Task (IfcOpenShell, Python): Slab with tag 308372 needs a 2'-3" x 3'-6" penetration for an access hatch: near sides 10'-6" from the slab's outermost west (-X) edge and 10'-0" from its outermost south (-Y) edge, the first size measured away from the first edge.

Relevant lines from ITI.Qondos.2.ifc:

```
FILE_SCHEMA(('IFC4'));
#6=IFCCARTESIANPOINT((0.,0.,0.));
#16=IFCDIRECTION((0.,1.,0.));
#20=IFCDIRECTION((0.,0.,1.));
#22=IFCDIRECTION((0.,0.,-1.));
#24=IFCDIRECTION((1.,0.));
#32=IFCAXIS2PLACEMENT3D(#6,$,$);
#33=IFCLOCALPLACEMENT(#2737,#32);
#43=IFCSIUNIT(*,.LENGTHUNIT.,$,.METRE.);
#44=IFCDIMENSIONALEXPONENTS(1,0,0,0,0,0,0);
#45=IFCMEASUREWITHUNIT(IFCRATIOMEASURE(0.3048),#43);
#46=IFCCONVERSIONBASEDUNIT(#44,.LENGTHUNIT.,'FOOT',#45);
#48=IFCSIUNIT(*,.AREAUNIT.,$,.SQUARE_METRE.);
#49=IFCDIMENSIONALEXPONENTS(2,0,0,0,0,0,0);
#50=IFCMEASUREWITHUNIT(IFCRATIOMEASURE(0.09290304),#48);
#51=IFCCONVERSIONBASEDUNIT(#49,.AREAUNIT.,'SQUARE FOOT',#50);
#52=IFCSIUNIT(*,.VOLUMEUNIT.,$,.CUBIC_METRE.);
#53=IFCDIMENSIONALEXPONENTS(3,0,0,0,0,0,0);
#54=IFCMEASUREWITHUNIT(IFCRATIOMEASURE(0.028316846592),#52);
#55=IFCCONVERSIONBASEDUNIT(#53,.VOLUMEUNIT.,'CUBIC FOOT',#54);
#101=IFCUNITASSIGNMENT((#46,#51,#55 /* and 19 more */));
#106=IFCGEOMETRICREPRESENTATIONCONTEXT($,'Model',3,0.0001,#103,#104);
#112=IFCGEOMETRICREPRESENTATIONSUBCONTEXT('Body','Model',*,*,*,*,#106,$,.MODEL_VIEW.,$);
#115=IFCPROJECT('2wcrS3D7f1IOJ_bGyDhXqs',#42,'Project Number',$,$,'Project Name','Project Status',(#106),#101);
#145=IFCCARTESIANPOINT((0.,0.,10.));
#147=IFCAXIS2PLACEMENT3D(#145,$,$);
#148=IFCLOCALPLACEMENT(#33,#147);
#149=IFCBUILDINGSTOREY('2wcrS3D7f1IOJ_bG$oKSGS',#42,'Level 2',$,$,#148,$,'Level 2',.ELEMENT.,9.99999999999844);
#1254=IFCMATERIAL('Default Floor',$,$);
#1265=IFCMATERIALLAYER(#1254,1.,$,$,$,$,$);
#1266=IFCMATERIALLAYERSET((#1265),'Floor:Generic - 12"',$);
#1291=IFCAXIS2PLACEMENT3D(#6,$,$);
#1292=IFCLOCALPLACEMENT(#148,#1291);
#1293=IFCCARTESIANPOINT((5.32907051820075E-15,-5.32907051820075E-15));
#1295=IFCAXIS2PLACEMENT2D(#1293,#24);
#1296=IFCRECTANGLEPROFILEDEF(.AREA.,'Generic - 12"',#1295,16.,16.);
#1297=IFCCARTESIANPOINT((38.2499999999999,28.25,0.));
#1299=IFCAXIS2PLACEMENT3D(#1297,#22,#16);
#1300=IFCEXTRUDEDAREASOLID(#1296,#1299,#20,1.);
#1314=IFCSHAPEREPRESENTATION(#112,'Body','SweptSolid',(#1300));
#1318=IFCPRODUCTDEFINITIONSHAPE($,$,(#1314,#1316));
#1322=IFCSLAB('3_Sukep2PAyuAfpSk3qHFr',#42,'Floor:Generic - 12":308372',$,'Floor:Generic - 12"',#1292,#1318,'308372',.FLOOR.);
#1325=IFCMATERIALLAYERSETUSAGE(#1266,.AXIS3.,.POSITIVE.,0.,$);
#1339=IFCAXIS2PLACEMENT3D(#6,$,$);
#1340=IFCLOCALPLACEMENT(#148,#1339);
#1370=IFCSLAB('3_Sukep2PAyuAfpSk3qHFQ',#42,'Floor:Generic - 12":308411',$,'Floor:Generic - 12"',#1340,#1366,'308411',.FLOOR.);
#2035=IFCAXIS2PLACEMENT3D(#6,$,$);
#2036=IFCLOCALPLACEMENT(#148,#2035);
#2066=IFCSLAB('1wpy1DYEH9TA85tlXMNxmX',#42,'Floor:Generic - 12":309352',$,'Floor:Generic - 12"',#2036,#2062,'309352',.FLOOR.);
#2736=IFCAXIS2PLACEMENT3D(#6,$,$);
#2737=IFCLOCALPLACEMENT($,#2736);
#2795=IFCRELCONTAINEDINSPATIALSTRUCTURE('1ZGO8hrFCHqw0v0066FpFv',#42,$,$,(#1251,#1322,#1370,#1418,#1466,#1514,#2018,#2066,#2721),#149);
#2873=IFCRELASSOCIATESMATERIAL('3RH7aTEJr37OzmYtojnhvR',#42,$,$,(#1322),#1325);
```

```python
import numpy as np
import ifcopenshell
import ifcopenshell.api.feature
import ifcopenshell.api.geometry
import ifcopenshell.api.root
import ifcopenshell.geom
import ifcopenshell.util.placement
import ifcopenshell.util.representation
import ifcopenshell.util.shape
import ifcopenshell.util.unit

model = ifcopenshell.open("ITI.Qondos.2.ifc")
unit_scale = ifcopenshell.util.unit.calculate_unit_scale(model)
settings = ifcopenshell.geom.settings()


def volume(element):
    """Net volume in cubic metres, openings subtracted."""
    shape = ifcopenshell.geom.create_shape(settings, element)
    return ifcopenshell.util.shape.get_volume(shape.geometry)


slab = model.by_guid("3_Sukep2PAyuAfpSk3qHFr")
before = volume(slab)

# Extent in the slab's own axes, in metres. The edges named are its -X and -Y sides.
slab_shape = ifcopenshell.geom.create_shape(settings, slab)
vertices = ifcopenshell.util.shape.get_vertices(slab_shape.geometry)
x_min, y_min, bottom = vertices.min(axis=0)
top = vertices[:, 2].max()

opening = ifcopenshell.api.root.create_entity(model, ifc_class="IfcOpeningElement", name="Access hatch opening", predefined_type="OPENING")
context = ifcopenshell.util.representation.get_context(model, "Model", "Body", "MODEL_VIEW")
width, depth = 0.6858, 1.0668
outline = [(0.0, 0.0), (width, 0.0), (width, depth), (0.0, depth), (0.0, 0.0)]
# Overshoot both faces by 50 mm so the cut is clean.
shape = ifcopenshell.api.geometry.add_slab_representation(
    model, context=context, depth=top - bottom + 0.1, polyline=outline
)
ifcopenshell.api.geometry.assign_representation(model, product=opening, representation=shape)

matrix = ifcopenshell.util.placement.get_local_placement(slab.ObjectPlacement)
matrix[:, 3] = matrix @ np.append(np.array([x_min + 3.2004, y_min + 3.048, bottom - 0.05]) / unit_scale, 1.0)
ifcopenshell.api.geometry.edit_object_placement(model, product=opening, matrix=matrix, is_si=False)
ifcopenshell.api.feature.add_feature(model, feature=opening, element=slab)

after = volume(slab)

print(f"slab volume {before:.3f} -> {after:.3f} m3")

model.write("ITI.Qondos.2-out.ifc")
```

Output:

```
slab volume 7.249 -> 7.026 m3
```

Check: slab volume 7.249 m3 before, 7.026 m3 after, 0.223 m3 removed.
